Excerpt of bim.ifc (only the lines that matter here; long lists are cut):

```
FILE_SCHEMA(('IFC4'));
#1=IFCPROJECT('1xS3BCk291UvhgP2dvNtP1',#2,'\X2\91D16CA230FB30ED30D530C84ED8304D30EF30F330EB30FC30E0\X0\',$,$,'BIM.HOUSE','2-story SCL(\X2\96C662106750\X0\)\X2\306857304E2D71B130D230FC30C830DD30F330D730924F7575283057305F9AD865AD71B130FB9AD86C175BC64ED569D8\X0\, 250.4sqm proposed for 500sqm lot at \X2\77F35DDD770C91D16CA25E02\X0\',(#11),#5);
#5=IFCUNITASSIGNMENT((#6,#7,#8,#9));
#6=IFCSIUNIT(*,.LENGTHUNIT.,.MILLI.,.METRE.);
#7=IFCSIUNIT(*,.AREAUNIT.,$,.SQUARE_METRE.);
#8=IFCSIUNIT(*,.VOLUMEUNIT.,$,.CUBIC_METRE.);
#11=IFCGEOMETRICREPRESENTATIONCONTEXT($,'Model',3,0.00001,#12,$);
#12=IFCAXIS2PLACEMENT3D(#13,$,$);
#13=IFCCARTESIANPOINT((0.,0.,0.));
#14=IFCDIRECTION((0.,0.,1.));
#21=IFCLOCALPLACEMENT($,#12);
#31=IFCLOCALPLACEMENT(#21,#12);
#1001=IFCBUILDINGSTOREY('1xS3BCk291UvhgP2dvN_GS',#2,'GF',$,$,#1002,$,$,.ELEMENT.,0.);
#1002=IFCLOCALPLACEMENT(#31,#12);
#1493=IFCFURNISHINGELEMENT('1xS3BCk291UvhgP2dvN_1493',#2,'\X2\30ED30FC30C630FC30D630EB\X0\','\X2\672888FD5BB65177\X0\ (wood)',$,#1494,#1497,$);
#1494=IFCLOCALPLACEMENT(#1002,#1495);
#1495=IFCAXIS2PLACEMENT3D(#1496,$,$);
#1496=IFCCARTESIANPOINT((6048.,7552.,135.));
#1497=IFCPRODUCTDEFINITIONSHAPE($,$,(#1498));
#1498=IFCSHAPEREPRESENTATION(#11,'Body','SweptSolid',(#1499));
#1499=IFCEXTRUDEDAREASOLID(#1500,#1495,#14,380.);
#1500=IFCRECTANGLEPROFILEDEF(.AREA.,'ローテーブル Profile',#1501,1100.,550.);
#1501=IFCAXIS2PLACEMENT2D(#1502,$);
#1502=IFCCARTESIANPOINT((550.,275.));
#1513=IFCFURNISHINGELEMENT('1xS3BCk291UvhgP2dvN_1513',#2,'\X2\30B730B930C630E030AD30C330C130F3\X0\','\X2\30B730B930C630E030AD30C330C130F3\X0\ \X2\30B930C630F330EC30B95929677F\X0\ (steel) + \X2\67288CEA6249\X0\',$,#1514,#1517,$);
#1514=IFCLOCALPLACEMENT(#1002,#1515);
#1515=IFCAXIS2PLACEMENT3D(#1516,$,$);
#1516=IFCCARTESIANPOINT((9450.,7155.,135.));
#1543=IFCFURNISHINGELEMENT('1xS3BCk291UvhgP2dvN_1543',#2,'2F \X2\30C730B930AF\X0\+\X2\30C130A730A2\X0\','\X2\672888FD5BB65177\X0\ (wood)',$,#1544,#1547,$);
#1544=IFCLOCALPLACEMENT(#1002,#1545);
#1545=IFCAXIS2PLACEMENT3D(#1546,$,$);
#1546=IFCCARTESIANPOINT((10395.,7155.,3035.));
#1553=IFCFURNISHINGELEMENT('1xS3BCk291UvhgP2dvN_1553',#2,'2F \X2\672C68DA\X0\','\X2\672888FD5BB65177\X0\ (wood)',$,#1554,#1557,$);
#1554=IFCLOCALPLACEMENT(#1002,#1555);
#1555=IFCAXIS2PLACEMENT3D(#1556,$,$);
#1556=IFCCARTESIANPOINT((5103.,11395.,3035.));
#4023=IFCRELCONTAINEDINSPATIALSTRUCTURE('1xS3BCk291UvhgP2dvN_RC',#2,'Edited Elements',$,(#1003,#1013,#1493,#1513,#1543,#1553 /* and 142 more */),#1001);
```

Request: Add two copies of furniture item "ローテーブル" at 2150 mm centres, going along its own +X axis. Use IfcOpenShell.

```python
import ifcopenshell
import ifcopenshell.api.geometry
import ifcopenshell.api.root
import ifcopenshell.util.element
import ifcopenshell.util.placement

model = ifcopenshell.open("bim.ifc")


def reuse_history(source, copy):
    """copy_class also copies each property set's owner history, people and application; keep the originals."""
    for rel in copy.IsDefinedBy:
        if rel.is_a("IfcRelDefinesByProperties") and (history := rel.RelatingPropertyDefinition.OwnerHistory):
            rel.RelatingPropertyDefinition.OwnerHistory = source.OwnerHistory
            ifcopenshell.util.element.remove_deep2(model, history)


source = model.by_guid("1xS3BCk291UvhgP2dvN_1493")
base = ifcopenshell.util.placement.get_local_placement(source.ObjectPlacement)
step = base[:3, 0] * 2150.0

for i in range(1, 3):
    copy = ifcopenshell.api.root.copy_class(model, product=source)
    copy.Representation = ifcopenshell.util.element.copy_deep(
        model, source.Representation, exclude=["IfcGeometricRepresentationContext", "IfcRepresentationMap"]
    )
    reuse_history(source, copy)
    matrix = base.copy()
    matrix[:3, 3] += i * step
    print("added at", matrix[:3, 3].round(3) + 0.0)
    ifcopenshell.api.geometry.edit_object_placement(model, product=copy, matrix=matrix, is_si=False)

model.write("bim_edited.ifc")
```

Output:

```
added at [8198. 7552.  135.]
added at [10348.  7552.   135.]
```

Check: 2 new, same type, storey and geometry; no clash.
